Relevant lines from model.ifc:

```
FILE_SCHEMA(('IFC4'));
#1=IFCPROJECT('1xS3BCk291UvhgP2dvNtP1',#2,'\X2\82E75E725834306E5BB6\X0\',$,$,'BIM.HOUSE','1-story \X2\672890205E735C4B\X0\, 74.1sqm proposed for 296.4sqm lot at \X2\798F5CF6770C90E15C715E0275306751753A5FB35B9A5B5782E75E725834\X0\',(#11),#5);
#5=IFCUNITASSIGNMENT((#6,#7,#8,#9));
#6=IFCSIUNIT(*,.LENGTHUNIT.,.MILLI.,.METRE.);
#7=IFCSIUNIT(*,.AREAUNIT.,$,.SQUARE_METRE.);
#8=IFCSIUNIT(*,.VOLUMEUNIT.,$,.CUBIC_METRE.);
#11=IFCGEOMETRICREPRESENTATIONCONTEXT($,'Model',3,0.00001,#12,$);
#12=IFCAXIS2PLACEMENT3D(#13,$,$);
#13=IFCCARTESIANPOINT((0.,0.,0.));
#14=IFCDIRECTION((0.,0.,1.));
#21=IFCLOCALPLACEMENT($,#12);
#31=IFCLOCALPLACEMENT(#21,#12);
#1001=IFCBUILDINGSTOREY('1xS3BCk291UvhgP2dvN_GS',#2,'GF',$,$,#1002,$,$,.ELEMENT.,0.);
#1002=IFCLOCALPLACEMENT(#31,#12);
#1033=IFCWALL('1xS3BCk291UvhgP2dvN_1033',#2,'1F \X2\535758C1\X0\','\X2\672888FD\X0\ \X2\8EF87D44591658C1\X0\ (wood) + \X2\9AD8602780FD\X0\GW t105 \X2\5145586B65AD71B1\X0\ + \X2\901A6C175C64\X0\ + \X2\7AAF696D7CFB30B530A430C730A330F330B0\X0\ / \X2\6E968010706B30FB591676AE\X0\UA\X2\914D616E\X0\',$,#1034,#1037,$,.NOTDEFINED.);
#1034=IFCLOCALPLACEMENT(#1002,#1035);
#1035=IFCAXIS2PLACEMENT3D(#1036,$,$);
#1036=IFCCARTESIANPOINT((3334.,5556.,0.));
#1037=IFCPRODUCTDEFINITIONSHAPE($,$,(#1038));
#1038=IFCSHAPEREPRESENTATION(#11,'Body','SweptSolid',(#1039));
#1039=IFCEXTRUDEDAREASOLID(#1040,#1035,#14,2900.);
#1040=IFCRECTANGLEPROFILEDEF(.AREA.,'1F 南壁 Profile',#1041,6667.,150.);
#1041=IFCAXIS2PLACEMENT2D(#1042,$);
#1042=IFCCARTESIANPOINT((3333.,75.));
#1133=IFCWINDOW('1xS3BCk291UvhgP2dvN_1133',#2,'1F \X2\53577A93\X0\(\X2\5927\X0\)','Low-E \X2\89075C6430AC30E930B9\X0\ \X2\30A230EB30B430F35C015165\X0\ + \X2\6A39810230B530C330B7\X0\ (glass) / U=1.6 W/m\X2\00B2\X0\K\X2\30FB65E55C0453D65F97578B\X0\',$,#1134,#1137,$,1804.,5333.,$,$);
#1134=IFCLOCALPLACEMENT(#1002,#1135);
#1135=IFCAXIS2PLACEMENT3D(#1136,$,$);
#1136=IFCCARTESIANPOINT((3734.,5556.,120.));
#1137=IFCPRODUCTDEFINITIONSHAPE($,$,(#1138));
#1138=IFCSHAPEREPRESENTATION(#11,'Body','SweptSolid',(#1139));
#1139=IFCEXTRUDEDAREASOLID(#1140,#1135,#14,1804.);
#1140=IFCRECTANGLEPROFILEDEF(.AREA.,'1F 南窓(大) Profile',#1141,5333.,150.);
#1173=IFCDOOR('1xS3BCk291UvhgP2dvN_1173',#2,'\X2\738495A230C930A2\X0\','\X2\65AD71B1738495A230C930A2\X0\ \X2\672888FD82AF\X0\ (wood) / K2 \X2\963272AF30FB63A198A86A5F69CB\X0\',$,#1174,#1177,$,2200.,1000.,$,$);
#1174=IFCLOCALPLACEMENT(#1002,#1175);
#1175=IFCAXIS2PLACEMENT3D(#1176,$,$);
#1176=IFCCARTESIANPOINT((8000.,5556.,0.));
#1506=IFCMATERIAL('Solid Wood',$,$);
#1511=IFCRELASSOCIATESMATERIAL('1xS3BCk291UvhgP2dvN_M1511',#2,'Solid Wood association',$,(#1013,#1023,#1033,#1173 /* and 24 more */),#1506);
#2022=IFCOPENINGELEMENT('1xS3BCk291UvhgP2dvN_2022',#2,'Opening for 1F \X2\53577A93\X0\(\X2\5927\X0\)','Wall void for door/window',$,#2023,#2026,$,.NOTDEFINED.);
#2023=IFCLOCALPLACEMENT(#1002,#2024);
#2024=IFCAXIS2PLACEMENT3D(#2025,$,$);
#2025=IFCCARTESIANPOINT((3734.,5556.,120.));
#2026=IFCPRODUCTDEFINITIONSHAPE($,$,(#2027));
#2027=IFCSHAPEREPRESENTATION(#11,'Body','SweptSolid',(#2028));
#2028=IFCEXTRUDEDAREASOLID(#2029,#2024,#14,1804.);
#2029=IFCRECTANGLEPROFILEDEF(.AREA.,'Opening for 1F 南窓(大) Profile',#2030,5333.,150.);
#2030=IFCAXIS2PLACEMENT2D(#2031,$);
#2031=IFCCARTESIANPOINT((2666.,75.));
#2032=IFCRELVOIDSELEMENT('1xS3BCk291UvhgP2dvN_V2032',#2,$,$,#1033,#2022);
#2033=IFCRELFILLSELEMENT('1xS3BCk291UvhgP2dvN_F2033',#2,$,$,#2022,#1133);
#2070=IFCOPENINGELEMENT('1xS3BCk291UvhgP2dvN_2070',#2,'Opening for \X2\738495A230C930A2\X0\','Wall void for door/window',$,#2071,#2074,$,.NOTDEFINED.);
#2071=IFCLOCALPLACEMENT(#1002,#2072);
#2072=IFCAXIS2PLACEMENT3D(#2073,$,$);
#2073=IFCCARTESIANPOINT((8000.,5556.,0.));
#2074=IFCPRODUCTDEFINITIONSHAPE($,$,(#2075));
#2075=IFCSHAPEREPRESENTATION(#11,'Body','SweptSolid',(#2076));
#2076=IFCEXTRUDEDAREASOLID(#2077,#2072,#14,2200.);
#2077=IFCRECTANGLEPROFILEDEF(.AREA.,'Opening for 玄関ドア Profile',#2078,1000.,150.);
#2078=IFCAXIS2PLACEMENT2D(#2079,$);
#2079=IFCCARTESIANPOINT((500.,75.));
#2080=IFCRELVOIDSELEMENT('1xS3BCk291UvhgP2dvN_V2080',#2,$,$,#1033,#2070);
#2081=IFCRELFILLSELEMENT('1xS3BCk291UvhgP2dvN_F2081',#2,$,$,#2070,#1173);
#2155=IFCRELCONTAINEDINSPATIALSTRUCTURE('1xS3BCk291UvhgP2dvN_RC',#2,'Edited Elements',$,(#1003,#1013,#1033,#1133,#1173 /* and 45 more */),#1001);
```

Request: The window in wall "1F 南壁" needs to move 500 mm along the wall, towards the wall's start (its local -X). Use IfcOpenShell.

```python
import ifcopenshell
import ifcopenshell.api.geometry
import ifcopenshell.util.placement
import ifcopenshell.util.unit

model = ifcopenshell.open("model.ifc")
unit_scale = ifcopenshell.util.unit.calculate_unit_scale(model)

window = model.by_id(1133)
opening = window.FillsVoids[0].RelatingOpeningElement
wall = opening.VoidsElements[0].RelatingBuildingElement

wall_matrix = ifcopenshell.util.placement.get_local_placement(wall.ObjectPlacement)
shift = wall_matrix[:3, 0] * -0.5 / unit_scale
before = ifcopenshell.util.placement.get_local_placement(window.ObjectPlacement)[:3, 3].copy()

# The window is not placed relative to its opening, so move both.
for product in (opening, window):
    matrix = ifcopenshell.util.placement.get_local_placement(product.ObjectPlacement)
    matrix[:3, 3] += shift
    ifcopenshell.api.geometry.edit_object_placement(model, product=product, matrix=matrix, is_si=False)

after = ifcopenshell.util.placement.get_local_placement(window.ObjectPlacement)[:3, 3]
print("window moved by", (after - before).round(3) + 0.0)

model.write("model_updated.ifc")
```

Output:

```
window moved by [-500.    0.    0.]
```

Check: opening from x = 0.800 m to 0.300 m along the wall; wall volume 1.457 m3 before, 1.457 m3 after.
